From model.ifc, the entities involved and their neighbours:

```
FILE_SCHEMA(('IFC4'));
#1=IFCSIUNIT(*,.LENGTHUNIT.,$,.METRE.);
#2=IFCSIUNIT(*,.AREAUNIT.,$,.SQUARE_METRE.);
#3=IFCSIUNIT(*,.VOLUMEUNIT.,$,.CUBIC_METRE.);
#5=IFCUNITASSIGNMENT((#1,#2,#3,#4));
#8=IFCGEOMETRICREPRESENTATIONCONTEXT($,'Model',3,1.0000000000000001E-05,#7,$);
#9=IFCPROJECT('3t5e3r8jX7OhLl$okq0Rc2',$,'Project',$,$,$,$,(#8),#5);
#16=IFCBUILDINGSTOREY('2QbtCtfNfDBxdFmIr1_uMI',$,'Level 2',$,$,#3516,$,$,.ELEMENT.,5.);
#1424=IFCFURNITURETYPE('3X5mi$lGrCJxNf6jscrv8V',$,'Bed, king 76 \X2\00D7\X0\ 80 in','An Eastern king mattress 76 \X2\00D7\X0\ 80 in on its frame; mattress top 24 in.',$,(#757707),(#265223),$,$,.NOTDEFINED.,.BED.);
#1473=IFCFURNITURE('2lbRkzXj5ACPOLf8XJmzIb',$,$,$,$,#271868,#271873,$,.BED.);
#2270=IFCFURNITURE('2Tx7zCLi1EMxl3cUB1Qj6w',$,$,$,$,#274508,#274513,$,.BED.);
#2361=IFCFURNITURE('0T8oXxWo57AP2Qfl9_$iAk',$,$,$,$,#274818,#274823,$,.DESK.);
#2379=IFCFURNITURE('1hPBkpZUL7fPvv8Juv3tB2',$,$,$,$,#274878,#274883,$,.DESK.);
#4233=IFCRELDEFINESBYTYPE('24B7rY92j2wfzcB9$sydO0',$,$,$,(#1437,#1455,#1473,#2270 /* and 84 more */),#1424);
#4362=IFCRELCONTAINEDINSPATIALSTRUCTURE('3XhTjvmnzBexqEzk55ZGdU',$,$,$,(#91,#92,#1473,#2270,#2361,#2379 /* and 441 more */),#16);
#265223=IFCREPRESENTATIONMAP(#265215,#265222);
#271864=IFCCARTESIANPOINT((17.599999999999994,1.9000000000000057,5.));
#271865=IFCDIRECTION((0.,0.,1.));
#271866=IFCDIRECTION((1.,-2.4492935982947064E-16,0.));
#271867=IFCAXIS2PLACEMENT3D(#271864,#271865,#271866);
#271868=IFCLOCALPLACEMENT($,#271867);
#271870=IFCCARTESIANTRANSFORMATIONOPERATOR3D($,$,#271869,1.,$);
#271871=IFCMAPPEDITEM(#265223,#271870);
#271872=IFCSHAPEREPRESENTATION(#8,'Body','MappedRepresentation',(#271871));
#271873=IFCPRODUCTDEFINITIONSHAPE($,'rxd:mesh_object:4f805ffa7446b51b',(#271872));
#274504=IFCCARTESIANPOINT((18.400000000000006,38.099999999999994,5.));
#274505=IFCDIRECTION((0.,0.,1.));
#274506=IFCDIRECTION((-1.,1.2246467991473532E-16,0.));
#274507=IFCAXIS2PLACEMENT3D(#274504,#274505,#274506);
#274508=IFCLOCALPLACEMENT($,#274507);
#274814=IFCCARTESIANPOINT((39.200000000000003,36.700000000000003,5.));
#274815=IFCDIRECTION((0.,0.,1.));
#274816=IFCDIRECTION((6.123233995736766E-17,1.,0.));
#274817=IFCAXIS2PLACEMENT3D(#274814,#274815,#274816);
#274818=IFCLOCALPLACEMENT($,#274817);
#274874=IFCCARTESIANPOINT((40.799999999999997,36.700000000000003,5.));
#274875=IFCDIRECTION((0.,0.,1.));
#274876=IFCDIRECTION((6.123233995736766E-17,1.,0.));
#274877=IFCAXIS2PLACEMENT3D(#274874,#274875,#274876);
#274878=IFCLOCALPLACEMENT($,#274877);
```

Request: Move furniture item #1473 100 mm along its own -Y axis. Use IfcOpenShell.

```python
import ifcopenshell
import ifcopenshell.api.geometry
import ifcopenshell.util.placement
import ifcopenshell.util.unit

model = ifcopenshell.open("model.ifc")
unit_scale = ifcopenshell.util.unit.calculate_unit_scale(model)

item = model.by_guid("2lbRkzXj5ACPOLf8XJmzIb")
matrix = ifcopenshell.util.placement.get_local_placement(item.ObjectPlacement)
matrix[:3, 3] -= matrix[:3, 1] * 0.1 / unit_scale
ifcopenshell.api.geometry.edit_object_placement(model, product=item, matrix=matrix, is_si=False)

print(ifcopenshell.util.placement.get_local_placement(item.ObjectPlacement).round(3) + 0.0)

model.write("model_rev.ifc")
```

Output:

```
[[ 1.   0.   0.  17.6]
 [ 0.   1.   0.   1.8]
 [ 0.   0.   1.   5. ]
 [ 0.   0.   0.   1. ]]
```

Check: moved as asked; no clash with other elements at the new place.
